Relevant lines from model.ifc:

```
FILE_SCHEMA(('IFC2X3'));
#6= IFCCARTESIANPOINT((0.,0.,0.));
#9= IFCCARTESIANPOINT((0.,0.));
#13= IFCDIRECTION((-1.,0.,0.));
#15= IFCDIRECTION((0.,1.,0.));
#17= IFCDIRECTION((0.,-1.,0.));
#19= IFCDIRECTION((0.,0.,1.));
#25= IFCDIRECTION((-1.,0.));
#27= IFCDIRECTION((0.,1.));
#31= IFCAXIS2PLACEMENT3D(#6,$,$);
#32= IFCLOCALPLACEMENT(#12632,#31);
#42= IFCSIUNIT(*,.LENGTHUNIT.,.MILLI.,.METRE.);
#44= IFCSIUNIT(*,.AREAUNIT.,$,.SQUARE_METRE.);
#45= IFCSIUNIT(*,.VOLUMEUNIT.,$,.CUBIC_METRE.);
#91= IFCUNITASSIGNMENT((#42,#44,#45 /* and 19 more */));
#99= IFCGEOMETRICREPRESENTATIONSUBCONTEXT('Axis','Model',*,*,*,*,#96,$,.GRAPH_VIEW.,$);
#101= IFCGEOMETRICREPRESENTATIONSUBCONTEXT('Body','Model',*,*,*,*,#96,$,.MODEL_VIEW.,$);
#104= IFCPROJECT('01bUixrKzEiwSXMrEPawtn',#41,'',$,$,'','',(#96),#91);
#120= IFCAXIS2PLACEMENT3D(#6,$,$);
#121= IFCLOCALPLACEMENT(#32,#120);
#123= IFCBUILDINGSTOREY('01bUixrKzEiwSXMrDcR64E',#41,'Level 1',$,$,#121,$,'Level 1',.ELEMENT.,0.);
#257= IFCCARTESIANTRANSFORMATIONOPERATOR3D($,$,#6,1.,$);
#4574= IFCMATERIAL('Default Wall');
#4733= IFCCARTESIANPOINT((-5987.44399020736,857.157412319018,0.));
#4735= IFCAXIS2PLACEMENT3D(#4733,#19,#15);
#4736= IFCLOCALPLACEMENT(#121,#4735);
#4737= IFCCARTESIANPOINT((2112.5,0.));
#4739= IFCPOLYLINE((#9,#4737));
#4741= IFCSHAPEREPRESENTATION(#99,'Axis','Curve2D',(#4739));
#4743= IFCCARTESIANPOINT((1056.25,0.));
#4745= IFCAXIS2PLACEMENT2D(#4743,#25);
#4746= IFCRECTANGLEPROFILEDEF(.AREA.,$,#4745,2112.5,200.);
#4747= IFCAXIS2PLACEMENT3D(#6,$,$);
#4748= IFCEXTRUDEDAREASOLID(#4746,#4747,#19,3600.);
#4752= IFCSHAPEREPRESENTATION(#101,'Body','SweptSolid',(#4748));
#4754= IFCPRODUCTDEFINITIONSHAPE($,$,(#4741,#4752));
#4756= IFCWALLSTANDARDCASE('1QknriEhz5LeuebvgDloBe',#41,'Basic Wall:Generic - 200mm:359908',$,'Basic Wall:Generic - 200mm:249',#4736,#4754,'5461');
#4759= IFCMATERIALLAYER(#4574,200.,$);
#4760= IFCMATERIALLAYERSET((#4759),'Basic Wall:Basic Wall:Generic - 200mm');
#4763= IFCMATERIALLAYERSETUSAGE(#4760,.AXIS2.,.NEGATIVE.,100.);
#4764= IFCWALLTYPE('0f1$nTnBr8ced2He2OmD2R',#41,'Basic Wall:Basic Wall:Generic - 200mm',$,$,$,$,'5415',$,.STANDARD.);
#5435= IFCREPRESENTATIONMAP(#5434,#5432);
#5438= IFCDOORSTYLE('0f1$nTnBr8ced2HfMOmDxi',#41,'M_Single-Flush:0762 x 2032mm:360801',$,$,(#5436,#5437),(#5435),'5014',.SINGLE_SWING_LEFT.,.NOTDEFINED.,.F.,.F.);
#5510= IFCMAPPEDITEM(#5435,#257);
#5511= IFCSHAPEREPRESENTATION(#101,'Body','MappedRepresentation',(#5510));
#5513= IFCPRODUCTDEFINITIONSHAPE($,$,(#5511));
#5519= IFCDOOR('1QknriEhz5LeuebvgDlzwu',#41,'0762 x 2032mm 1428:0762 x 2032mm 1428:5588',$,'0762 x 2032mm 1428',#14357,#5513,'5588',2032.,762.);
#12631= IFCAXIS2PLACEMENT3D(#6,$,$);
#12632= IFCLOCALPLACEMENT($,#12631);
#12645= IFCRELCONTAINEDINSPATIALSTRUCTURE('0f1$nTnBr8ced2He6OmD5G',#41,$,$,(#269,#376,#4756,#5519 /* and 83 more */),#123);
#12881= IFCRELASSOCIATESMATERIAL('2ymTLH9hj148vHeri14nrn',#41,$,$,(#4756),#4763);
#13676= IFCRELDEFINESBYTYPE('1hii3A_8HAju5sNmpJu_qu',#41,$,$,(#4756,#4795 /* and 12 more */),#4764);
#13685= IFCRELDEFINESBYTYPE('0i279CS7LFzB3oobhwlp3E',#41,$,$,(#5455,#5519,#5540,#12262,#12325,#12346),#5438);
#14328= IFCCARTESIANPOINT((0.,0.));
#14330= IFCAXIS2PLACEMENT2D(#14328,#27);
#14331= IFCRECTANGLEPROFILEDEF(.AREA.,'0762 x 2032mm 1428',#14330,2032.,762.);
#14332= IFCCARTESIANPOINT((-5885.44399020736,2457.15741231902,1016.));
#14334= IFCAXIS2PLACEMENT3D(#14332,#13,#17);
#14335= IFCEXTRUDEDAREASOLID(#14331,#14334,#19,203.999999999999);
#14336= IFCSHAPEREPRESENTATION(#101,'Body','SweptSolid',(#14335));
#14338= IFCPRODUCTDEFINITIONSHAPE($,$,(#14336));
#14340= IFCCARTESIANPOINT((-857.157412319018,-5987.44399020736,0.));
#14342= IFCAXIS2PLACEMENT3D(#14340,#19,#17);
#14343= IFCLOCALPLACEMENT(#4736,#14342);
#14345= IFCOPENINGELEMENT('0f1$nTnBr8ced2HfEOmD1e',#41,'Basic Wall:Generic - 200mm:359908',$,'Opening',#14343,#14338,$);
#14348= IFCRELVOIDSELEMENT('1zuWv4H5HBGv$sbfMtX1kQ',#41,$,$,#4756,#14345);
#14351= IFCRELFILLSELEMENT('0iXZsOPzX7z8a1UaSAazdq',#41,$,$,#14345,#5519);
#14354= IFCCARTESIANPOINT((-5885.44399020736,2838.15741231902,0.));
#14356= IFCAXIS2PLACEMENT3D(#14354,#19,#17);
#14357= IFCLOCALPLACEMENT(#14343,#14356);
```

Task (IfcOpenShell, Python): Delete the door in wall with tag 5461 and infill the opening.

```python
import ifcopenshell
import ifcopenshell.api.feature
import ifcopenshell.api.root
import ifcopenshell.geom
import ifcopenshell.util.shape

model = ifcopenshell.open("model.ifc")
settings = ifcopenshell.geom.settings()


def volume(element):
    """Net volume in cubic metres, openings subtracted."""
    shape = ifcopenshell.geom.create_shape(settings, element)
    return ifcopenshell.util.shape.get_volume(shape.geometry)


door = model.by_guid("1QknriEhz5LeuebvgDlzwu")
opening = door.FillsVoids[0].RelatingOpeningElement
wall = opening.VoidsElements[0].RelatingBuildingElement
before = volume(wall)

ifcopenshell.api.root.remove_product(model, product=door)
ifcopenshell.api.feature.remove_feature(model, feature=opening)

after = volume(wall)

print(f"wall volume {before:.3f} -> {after:.3f} m3")

model.write("model_updated.ifc")
```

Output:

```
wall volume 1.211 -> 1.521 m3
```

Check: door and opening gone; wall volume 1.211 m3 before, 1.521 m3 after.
